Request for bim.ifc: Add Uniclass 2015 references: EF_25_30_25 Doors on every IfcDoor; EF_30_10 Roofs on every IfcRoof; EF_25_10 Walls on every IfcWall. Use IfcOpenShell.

First a look at what the model holds.

```python
import ifcopenshell

model = ifcopenshell.open("bim.ifc")
print(model.schema)
print("classifications:", [c.Name for c in model.by_type("IfcClassification")])
for ifc_class in ("IfcDoor", "IfcRoof", "IfcStair", "IfcWall", "IfcWindow"):
    print(ifc_class, len(model.by_type(ifc_class)))
```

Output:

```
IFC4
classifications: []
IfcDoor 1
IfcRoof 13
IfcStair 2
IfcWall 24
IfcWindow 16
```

```python
import ifcopenshell
import ifcopenshell.api.classification

model = ifcopenshell.open("bim.ifc")

system = ifcopenshell.api.classification.add_classification(model, classification="Uniclass 2015")

codes = {
    "IfcDoor": ("EF_25_30_25", "Doors"),
    "IfcRoof": ("EF_30_10", "Roofs"),
    "IfcWall": ("EF_25_10", "Walls"),
}
for ifc_class, (code, name) in codes.items():
    products = model.by_type(ifc_class)
    ifcopenshell.api.classification.add_reference(
        model, products=products, classification=system, identification=code, name=name
    )
    print(code, len(products))

model.write("bim_v2.ifc")
```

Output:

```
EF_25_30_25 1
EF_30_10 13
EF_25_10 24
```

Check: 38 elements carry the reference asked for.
